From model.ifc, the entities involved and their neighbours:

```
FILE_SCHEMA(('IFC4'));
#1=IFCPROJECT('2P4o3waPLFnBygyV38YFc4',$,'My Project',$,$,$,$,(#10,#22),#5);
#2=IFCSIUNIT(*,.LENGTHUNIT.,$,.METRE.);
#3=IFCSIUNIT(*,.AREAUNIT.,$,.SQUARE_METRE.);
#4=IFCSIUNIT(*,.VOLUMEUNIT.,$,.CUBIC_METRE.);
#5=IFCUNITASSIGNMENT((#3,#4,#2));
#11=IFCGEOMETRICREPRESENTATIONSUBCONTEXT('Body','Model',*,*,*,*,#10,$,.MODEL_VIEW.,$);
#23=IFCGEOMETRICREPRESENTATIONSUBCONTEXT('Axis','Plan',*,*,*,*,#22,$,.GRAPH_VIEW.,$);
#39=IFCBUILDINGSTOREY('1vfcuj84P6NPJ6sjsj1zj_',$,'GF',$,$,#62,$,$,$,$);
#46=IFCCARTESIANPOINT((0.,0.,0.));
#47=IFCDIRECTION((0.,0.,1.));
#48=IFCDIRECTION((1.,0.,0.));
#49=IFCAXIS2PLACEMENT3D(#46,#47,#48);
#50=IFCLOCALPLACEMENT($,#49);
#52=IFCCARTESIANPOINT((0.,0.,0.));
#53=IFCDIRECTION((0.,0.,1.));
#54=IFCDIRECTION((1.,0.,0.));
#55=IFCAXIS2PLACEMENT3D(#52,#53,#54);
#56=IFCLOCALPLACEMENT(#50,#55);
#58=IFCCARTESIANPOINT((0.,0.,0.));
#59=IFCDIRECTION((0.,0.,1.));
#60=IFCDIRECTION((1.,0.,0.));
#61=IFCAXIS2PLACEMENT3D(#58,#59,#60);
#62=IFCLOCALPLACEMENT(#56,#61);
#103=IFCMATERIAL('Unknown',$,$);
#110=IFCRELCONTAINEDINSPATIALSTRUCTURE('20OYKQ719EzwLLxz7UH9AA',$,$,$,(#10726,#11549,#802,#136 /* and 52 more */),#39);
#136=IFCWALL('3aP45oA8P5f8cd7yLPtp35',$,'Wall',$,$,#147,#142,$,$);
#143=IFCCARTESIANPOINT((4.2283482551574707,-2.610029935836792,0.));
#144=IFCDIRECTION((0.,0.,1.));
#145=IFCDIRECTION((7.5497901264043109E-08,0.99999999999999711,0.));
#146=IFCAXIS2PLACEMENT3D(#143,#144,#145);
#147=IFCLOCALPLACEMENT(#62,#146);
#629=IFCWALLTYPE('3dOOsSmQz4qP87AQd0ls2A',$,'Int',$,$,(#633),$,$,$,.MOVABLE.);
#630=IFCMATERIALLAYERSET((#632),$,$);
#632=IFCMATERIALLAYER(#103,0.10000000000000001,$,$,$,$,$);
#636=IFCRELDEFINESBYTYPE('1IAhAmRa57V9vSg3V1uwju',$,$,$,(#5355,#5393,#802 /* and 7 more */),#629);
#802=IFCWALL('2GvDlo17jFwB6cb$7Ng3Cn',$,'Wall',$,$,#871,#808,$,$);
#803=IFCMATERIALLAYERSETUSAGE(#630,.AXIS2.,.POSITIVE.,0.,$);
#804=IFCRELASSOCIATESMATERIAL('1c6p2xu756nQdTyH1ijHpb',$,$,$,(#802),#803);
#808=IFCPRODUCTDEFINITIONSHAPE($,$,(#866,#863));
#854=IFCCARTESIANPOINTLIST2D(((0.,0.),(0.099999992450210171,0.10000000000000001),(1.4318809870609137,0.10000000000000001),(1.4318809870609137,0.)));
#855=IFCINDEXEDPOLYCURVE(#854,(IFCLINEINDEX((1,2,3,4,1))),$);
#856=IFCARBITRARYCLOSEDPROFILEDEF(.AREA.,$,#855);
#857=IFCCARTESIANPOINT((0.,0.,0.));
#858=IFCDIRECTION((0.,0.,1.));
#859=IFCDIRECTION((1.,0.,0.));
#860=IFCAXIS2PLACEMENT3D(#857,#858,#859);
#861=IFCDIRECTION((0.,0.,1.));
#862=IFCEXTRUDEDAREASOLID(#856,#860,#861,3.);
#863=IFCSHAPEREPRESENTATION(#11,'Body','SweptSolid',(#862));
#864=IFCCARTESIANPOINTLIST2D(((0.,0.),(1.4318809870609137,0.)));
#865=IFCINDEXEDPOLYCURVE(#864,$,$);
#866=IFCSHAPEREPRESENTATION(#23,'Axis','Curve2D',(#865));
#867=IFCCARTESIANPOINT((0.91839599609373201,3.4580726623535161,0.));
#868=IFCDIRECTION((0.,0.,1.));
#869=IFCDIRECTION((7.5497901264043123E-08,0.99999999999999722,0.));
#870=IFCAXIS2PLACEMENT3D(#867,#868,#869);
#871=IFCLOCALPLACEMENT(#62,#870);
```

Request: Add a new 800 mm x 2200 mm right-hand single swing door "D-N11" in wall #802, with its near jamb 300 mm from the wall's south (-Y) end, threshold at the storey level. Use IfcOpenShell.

```python
import numpy as np
import ifcopenshell
import ifcopenshell.api.feature
import ifcopenshell.api.geometry
import ifcopenshell.api.root
import ifcopenshell.api.spatial
import ifcopenshell.geom
import ifcopenshell.util.element
import ifcopenshell.util.placement
import ifcopenshell.util.representation
import ifcopenshell.util.shape
import ifcopenshell.util.unit

model = ifcopenshell.open("model.ifc")
unit_scale = ifcopenshell.util.unit.calculate_unit_scale(model)
settings = ifcopenshell.geom.settings()


def volume(element):
    """Net volume in cubic metres, openings subtracted."""
    shape = ifcopenshell.geom.create_shape(settings, element)
    return ifcopenshell.util.shape.get_volume(shape.geometry)


wall = model.by_id(802)
storey = ifcopenshell.util.element.get_container(wall, ifc_class="IfcBuildingStorey")
context = ifcopenshell.util.representation.get_context(model, "Model", "Body", "MODEL_VIEW")
before = volume(wall)

width, height, from_end, sill = 0.8, 2.2, 0.3, 0.0  # metres

# The wall runs along its own X axis, and the end named is its -X end.
wall_shape = ifcopenshell.geom.create_shape(settings, wall)
x, y, z = ifcopenshell.util.shape.get_vertices(wall_shape.geometry).T
start = x.min() + from_end
face, thickness = float(y.min()), float(y.max() - y.min())
wall_matrix = ifcopenshell.util.placement.get_local_placement(wall.ObjectPlacement)
level = ifcopenshell.util.placement.get_local_placement(storey.ObjectPlacement)[2, 3]


def in_wall(x, y):
    """Placement at x, y metres in the wall's axes, at sill height."""
    matrix = wall_matrix.copy()
    matrix[:, 3] = wall_matrix @ np.array([x / unit_scale, y / unit_scale, 0.0, 1.0])
    matrix[2, 3] = level + sill / unit_scale
    return matrix


# Opening: a box that overshoots both wall faces by 50 mm.
opening = ifcopenshell.api.root.create_entity(model, ifc_class="IfcOpeningElement", predefined_type="OPENING")
box = ifcopenshell.api.geometry.add_wall_representation(
    model, context=context, length=width, height=height, thickness=thickness + 0.1
)
ifcopenshell.api.geometry.assign_representation(model, product=opening, representation=box)
ifcopenshell.api.geometry.edit_object_placement(model, product=opening, matrix=in_wall(start, face - 0.05), is_si=False)
ifcopenshell.api.feature.add_feature(model, feature=opening, element=wall)

door = ifcopenshell.api.root.create_entity(model, ifc_class="IfcDoor", name="D-N11", predefined_type="DOOR")
door.OverallWidth, door.OverallHeight = width / unit_scale, height / unit_scale
door.OperationType = "SINGLE_SWING_RIGHT"
body = ifcopenshell.api.geometry.add_door_representation(
    model,
    context=context,
    overall_width=door.OverallWidth,
    overall_height=door.OverallHeight,
    operation_type="SINGLE_SWING_RIGHT",
    lining_properties={"LiningDepth": thickness / unit_scale, "ThresholdDepth": thickness / unit_scale},
)
ifcopenshell.api.geometry.assign_representation(model, product=door, representation=body)
ifcopenshell.api.spatial.assign_container(model, products=[door], relating_structure=storey)
ifcopenshell.api.feature.add_filling(model, opening=opening, element=door)

# The lining spans the wall, so the door starts at the wall face.
ifcopenshell.api.geometry.edit_object_placement(model, product=door, matrix=in_wall(start, face), is_si=False)

after = volume(wall)

print(f"wall volume {before:.3f} -> {after:.3f} m3")

model.write("model_rev.ifc")
```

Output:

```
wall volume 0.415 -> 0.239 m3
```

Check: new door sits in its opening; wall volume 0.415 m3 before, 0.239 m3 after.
